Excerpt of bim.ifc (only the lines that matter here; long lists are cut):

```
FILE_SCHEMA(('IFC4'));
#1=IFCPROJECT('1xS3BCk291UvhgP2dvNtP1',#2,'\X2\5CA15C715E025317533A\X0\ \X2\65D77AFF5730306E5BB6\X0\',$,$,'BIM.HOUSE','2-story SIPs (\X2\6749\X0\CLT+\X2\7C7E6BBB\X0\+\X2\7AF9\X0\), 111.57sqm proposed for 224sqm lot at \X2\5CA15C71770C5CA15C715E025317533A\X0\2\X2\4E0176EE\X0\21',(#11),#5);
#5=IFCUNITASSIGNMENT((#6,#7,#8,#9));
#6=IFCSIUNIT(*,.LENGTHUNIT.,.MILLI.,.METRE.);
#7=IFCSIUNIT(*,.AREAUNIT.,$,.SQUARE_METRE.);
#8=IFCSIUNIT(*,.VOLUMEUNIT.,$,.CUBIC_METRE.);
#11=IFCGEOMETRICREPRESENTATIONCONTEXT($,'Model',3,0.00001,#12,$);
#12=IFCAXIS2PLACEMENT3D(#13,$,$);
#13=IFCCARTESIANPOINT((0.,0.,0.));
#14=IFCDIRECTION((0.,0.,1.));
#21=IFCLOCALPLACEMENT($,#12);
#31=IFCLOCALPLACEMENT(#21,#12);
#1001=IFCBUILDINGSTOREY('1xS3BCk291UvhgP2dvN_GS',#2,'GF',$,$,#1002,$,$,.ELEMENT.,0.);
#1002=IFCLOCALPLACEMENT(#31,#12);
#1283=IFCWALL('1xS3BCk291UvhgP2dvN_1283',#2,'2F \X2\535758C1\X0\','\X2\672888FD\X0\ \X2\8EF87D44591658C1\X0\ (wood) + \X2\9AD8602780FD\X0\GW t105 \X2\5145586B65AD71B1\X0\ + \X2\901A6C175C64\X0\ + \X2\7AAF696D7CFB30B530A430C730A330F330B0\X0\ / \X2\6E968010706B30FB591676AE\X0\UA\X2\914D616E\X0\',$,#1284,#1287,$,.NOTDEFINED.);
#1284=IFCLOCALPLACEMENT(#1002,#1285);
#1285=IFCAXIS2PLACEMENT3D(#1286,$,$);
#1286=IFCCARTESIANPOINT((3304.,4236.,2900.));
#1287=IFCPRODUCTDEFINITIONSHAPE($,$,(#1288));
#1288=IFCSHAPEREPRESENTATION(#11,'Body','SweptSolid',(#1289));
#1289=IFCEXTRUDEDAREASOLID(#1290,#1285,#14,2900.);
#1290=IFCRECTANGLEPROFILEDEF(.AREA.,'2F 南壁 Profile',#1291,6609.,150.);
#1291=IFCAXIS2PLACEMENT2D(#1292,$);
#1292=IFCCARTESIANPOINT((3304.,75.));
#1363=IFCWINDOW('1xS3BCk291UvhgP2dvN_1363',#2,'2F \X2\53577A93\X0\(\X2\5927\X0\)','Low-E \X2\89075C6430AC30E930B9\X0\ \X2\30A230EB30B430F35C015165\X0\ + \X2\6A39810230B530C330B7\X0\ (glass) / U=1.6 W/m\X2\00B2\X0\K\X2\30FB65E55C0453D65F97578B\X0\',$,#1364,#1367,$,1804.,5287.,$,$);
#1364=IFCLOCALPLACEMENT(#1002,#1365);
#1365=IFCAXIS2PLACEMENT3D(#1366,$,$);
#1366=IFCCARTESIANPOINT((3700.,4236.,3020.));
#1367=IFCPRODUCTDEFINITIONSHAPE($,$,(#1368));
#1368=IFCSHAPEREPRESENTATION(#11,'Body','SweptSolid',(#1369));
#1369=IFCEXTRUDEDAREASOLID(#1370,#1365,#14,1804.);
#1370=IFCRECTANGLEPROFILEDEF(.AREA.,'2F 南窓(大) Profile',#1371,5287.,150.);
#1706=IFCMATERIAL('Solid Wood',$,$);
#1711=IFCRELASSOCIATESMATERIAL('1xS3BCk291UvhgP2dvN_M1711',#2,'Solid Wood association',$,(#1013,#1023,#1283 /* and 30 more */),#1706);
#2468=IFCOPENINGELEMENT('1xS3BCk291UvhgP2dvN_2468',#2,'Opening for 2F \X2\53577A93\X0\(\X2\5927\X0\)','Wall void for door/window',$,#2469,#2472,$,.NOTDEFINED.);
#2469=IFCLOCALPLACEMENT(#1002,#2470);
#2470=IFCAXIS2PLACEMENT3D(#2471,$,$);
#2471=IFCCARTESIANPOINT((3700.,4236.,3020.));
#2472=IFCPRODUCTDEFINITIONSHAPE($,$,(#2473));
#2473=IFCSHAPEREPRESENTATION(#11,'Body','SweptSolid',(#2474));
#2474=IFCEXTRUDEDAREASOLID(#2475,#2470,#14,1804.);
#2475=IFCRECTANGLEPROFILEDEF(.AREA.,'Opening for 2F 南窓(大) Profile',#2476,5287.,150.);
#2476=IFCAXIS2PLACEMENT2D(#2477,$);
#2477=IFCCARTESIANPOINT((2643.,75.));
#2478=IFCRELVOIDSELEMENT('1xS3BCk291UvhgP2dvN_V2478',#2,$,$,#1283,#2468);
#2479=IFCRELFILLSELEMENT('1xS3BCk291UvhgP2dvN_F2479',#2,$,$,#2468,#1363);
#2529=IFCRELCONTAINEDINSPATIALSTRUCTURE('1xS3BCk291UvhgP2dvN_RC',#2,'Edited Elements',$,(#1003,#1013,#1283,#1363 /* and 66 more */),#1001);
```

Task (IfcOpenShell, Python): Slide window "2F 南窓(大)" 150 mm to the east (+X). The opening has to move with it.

```python
import ifcopenshell
import ifcopenshell.api.geometry
import ifcopenshell.util.placement
import ifcopenshell.util.unit

model = ifcopenshell.open("bim.ifc")
unit_scale = ifcopenshell.util.unit.calculate_unit_scale(model)

window = model.by_guid("1xS3BCk291UvhgP2dvN_1363")
opening = window.FillsVoids[0].RelatingOpeningElement
wall = opening.VoidsElements[0].RelatingBuildingElement

wall_matrix = ifcopenshell.util.placement.get_local_placement(wall.ObjectPlacement)
shift = wall_matrix[:3, 0] * 0.15 / unit_scale
before = ifcopenshell.util.placement.get_local_placement(window.ObjectPlacement)[:3, 3].copy()

# The window is not placed relative to its opening, so move both.
for product in (opening, window):
    matrix = ifcopenshell.util.placement.get_local_placement(product.ObjectPlacement)
    matrix[:3, 3] += shift
    ifcopenshell.api.geometry.edit_object_placement(model, product=product, matrix=matrix, is_si=False)

after = ifcopenshell.util.placement.get_local_placement(window.ObjectPlacement)[:3, 3]
print("window moved by", (after - before).round(3) + 0.0)

model.write("bim_rev.ifc")
```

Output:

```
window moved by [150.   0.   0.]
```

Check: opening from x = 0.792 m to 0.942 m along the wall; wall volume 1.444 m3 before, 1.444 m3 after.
